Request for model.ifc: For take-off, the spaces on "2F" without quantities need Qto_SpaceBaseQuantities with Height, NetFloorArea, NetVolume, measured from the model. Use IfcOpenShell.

First a look at what the model holds.

```python
import ifcopenshell
import ifcopenshell.util.element
import ifcopenshell.util.unit

model = ifcopenshell.open("model.ifc")
print(model.schema)
for unit_type in ("LENGTHUNIT", "AREAUNIT", "VOLUMEUNIT"):
    print(unit_type, ifcopenshell.util.unit.calculate_unit_scale(model, unit_type))
storey = next(s for s in model.by_type("IfcBuildingStorey") if s.Name == "2F")
spaces = [e for e in ifcopenshell.util.element.get_decomposition(storey) if e.is_a("IfcSpace")]
for e in sorted(spaces, key=lambda e: e.id()):
    print(e.id(), e.is_a(), e.Name, list(ifcopenshell.util.element.get_psets(e, qtos_only=True)), sep=" | ")
```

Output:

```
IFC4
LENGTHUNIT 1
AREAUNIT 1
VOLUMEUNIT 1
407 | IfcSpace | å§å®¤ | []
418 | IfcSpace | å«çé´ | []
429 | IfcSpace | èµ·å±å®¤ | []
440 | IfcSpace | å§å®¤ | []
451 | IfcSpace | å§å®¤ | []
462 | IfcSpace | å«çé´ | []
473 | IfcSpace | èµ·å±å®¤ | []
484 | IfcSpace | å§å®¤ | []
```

```python
import ifcopenshell
import ifcopenshell.api.pset
import ifcopenshell.geom
import ifcopenshell.util.element
import ifcopenshell.util.shape
import ifcopenshell.util.unit

model = ifcopenshell.open("model.ifc")
unit_scale = ifcopenshell.util.unit.calculate_unit_scale(model)
area_scale = ifcopenshell.util.unit.calculate_unit_scale(model, "AREAUNIT")
volume_scale = ifcopenshell.util.unit.calculate_unit_scale(model, "VOLUMEUNIT")
settings = ifcopenshell.geom.settings()

storey = next(s for s in model.by_type("IfcBuildingStorey") if s.Name == "2F")
spaces = [e for e in ifcopenshell.util.element.get_decomposition(storey) if e.is_a("IfcSpace")]

for e in sorted(spaces, key=lambda e: e.id()):
    if ifcopenshell.util.element.get_psets(e, qtos_only=True, should_inherit=False):
        continue
    # Geometry comes back in metres, in the element's own axes.
    shape = ifcopenshell.geom.create_shape(settings, e)
    values = {
        "Height": ifcopenshell.util.shape.get_z(shape.geometry) / unit_scale,
        "NetFloorArea": ifcopenshell.util.shape.get_footprint_area(shape.geometry) / area_scale,
        "NetVolume": ifcopenshell.util.shape.get_volume(shape.geometry) / volume_scale,
    }
    qto = ifcopenshell.api.pset.add_qto(model, product=e, name="Qto_SpaceBaseQuantities")
    ifcopenshell.api.pset.edit_qto(model, qto=qto, properties=values)
    print(e.id(), {k: round(v, 3) for k, v in values.items()})

model.write("model_rev.ifc")
```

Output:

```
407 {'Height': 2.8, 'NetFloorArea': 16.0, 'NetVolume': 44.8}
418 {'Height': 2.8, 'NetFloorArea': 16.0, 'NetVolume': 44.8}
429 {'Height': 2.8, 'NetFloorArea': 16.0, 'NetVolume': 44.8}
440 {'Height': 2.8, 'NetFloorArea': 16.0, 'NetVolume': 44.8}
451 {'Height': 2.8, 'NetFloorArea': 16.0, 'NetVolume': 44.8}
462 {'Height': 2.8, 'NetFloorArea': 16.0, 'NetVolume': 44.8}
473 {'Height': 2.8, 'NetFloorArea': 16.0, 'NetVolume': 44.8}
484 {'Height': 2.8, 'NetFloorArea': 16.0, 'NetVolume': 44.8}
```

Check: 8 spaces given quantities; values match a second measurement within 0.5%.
